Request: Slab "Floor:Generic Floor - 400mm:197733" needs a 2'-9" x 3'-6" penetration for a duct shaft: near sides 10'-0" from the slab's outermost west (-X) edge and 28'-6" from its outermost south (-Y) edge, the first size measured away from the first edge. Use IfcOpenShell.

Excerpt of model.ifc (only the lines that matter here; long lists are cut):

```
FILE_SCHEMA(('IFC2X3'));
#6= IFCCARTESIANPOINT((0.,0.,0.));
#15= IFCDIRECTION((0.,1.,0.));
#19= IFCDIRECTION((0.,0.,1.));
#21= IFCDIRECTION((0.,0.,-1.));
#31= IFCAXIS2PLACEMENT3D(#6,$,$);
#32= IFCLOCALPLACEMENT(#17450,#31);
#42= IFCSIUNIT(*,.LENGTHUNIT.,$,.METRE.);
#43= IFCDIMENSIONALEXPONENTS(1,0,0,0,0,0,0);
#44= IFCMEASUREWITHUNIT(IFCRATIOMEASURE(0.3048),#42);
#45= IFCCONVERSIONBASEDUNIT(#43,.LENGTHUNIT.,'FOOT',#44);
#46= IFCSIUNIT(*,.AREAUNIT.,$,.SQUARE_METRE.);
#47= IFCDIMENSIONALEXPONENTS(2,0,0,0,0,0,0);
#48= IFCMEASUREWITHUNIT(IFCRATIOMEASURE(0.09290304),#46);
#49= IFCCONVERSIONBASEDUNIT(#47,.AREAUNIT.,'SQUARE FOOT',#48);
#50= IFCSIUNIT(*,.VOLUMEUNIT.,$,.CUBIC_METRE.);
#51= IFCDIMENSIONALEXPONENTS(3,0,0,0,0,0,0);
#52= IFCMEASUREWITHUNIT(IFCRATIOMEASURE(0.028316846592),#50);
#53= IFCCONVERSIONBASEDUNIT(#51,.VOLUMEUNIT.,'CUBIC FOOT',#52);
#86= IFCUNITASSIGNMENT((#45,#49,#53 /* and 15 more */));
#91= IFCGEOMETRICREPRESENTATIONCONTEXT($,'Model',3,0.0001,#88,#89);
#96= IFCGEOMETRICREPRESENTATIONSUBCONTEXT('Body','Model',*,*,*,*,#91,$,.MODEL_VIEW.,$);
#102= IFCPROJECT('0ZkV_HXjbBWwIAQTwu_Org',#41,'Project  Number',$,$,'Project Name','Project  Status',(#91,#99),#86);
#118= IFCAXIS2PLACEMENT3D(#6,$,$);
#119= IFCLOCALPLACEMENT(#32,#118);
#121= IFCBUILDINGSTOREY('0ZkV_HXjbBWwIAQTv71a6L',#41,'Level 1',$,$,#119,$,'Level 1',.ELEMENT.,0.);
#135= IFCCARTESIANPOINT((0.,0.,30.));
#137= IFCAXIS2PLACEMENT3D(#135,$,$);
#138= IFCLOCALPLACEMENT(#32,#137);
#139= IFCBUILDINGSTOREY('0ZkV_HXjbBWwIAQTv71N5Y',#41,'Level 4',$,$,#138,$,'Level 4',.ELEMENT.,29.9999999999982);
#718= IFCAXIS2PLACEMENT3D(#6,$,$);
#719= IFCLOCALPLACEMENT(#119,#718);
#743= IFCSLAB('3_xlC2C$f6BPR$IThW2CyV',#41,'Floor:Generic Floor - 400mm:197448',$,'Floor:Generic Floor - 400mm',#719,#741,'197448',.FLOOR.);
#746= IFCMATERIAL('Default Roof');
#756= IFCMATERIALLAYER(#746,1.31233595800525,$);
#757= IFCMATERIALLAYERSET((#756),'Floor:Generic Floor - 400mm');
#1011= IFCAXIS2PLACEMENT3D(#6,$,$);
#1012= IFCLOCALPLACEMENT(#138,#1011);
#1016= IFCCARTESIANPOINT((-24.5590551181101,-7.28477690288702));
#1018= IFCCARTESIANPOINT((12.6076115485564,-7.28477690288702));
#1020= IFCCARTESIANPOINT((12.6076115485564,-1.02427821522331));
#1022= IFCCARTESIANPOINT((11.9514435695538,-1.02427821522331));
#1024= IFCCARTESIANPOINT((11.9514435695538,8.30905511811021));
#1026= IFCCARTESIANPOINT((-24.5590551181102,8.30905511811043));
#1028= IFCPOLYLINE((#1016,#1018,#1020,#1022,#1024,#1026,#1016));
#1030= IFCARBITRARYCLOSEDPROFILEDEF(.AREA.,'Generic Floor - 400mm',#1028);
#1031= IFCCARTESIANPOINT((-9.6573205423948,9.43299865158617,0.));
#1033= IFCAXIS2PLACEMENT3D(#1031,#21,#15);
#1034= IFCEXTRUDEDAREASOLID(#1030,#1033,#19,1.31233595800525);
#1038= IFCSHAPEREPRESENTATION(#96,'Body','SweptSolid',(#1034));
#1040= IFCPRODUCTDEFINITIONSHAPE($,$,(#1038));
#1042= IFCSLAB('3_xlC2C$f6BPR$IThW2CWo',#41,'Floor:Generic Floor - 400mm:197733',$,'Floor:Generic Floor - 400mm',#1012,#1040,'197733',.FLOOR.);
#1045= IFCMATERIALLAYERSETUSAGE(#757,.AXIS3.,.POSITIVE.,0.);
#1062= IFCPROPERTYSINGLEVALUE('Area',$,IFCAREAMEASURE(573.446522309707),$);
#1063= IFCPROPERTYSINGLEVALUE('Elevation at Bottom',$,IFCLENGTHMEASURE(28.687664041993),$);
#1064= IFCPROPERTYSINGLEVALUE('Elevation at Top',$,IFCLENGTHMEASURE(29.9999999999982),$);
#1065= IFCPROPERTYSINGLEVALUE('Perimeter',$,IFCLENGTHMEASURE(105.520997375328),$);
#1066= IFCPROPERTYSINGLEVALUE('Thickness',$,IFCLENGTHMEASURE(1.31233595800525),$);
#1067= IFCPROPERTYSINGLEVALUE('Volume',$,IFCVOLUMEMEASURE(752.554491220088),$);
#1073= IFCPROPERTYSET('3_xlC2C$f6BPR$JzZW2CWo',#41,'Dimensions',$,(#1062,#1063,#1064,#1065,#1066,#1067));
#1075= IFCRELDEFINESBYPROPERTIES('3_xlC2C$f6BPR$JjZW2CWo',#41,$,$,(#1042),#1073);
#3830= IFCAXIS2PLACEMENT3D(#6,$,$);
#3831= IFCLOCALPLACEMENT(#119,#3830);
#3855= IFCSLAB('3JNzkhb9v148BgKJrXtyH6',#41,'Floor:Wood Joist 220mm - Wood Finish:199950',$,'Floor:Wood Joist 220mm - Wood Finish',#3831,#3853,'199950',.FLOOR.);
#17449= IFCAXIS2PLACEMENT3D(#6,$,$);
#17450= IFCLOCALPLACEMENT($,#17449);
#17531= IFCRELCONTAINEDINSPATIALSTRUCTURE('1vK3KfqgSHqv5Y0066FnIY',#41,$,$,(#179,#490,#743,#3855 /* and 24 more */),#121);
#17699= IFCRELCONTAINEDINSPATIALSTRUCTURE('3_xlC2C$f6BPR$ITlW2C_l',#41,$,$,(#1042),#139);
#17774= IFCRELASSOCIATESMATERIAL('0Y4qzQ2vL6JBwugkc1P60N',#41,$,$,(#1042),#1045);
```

```python
import numpy as np
import ifcopenshell
import ifcopenshell.api.feature
import ifcopenshell.api.geometry
import ifcopenshell.api.pset
import ifcopenshell.api.root
import ifcopenshell.geom
import ifcopenshell.util.element
import ifcopenshell.util.placement
import ifcopenshell.util.representation
import ifcopenshell.util.shape
import ifcopenshell.util.unit

model = ifcopenshell.open("model.ifc")
unit_scale = ifcopenshell.util.unit.calculate_unit_scale(model)
area_scale = ifcopenshell.util.unit.calculate_unit_scale(model, "AREAUNIT")
volume_scale = ifcopenshell.util.unit.calculate_unit_scale(model, "VOLUMEUNIT")
settings = ifcopenshell.geom.settings()


def volume(element):
    """Net volume in cubic metres, openings subtracted."""
    shape = ifcopenshell.geom.create_shape(settings, element)
    return ifcopenshell.util.shape.get_volume(shape.geometry)


slab = model.by_id(1042)
before = volume(slab)

# Extent in the slab's own axes, in metres. The edges named are its -X and -Y sides.
slab_shape = ifcopenshell.geom.create_shape(settings, slab)
vertices = ifcopenshell.util.shape.get_vertices(slab_shape.geometry)
x_min, y_min, bottom = vertices.min(axis=0)
top = vertices[:, 2].max()

opening = ifcopenshell.api.root.create_entity(model, ifc_class="IfcOpeningElement", name="Duct shaft opening")
context = ifcopenshell.util.representation.get_context(model, "Model", "Body", "MODEL_VIEW")
width, depth = 0.8382, 1.0668
outline = [(0.0, 0.0), (width, 0.0), (width, depth), (0.0, depth), (0.0, 0.0)]
# Overshoot both faces by 50 mm so the cut is clean.
shape = ifcopenshell.api.geometry.add_slab_representation(
    model, context=context, depth=top - bottom + 0.1, polyline=outline
)
ifcopenshell.api.geometry.assign_representation(model, product=opening, representation=shape)

matrix = ifcopenshell.util.placement.get_local_placement(slab.ObjectPlacement)
matrix[:, 3] = matrix @ np.append(np.array([x_min + 3.048, y_min + 8.6868, bottom - 0.05]) / unit_scale, 1.0)
ifcopenshell.api.geometry.edit_object_placement(model, product=opening, matrix=matrix, is_si=False)
ifcopenshell.api.feature.add_feature(model, feature=opening, element=slab)

after = volume(slab)

# Update the slab's stored quantities.
pset = model.by_id(ifcopenshell.util.element.get_pset(slab, "Dimensions", should_inherit=False)["id"])
ifcopenshell.api.pset.edit_pset(model, pset=pset, properties={
    "Area": model.create_entity("IfcAreaMeasure", after / (top - bottom) / area_scale),
    "Volume": model.create_entity("IfcVolumeMeasure", after / volume_scale),
})

print(f"slab volume {before:.3f} -> {after:.3f} m3")

model.write("model_v2.ifc")
```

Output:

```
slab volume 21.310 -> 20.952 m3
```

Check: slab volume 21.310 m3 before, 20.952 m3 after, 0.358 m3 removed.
